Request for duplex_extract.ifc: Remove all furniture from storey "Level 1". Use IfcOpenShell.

First a look at what the model holds.

```python
import ifcopenshell
import ifcopenshell.util.element

model = ifcopenshell.open("duplex_extract.ifc")
print(model.schema)
storey = next(s for s in model.by_type("IfcBuildingStorey") if s.Name == "Level 1")
furniture = [e for e in ifcopenshell.util.element.get_decomposition(storey) if e.is_a("IfcFurnishingElement")]
seen = {}
for e in furniture:
    element_type = ifcopenshell.util.element.get_type(e)
    name = element_type.Name if element_type not in (None, e) else None
    seen[name] = seen.get(name, 0) + 1
for name, count in sorted(seen.items(), key=str):
    print(count, "x", name)
```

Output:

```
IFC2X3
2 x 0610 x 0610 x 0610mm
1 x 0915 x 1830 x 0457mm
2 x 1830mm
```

```python
import ifcopenshell
import ifcopenshell.api.root
import ifcopenshell.util.element

model = ifcopenshell.open("duplex_extract.ifc")

storey = next(s for s in model.by_type("IfcBuildingStorey") if s.Name == "Level 1")
furniture = [e for e in ifcopenshell.util.element.get_decomposition(storey) if e.is_a("IfcFurnishingElement")]

for e in furniture:
    ifcopenshell.api.root.remove_product(model, product=e)
print(len(furniture), "removed")

model.write("duplex_extract_edited.ifc")
```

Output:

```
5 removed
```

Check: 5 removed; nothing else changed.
